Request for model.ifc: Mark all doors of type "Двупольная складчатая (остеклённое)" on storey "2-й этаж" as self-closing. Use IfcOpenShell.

First a look at what the model holds.

```python
import ifcopenshell
import ifcopenshell.util.element

model = ifcopenshell.open("model.ifc")
print(model.schema)
storey = next(s for s in model.by_type("IfcBuildingStorey") if s.Name == "2-й этаж")
doors = [e for e in ifcopenshell.util.element.get_decomposition(storey) if e.is_a("IfcDoor")]
seen = {}
for e in doors:
    element_type = ifcopenshell.util.element.get_type(e)
    key = (element_type.Name if element_type != e and element_type else None, ifcopenshell.util.element.get_pset(e, "Pset_DoorCommon", "SelfClosing"))
    seen[key] = seen.get(key, 0) + 1
for (name, value), count in sorted(seen.items(), key=str):
    print(count, "x", name, "|", value)
```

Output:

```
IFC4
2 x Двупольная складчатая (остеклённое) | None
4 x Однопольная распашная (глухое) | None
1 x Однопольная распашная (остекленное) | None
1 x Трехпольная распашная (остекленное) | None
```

```python
import ifcopenshell
import ifcopenshell.api.pset
import ifcopenshell.util.element

model = ifcopenshell.open("model.ifc")

storey = next(s for s in model.by_type("IfcBuildingStorey") if s.Name == "2-й этаж")
doors = [e for e in ifcopenshell.util.element.get_decomposition(storey) if e.is_a("IfcDoor")]

count = 0
for e in doors:
    element_type = ifcopenshell.util.element.get_type(e)
    if element_type in (None, e) or element_type.Name != "Двупольная складчатая (остеклённое)":
        continue
    # add_pset returns the element's existing set when there is one.
    pset = ifcopenshell.api.pset.add_pset(model, product=e, name="Pset_DoorCommon")
    ifcopenshell.api.pset.edit_pset(model, pset=pset, properties={"SelfClosing": True})
    count += 1

print(count, "doors updated")

model.write("model_rev.ifc")
```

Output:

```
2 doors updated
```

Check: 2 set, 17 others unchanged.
